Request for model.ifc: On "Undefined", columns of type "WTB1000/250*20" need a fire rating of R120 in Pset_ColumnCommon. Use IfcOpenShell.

First a look at what the model holds.

```python
import ifcopenshell
import ifcopenshell.util.element

model = ifcopenshell.open("model.ifc")
print(model.schema)
storey = next(s for s in model.by_type("IfcBuildingStorey") if s.Name == "Undefined")
columns = [e for e in ifcopenshell.util.element.get_decomposition(storey) if e.is_a("IfcColumn")]
seen = {}
for e in columns:
    element_type = ifcopenshell.util.element.get_type(e)
    key = (element_type.Name if element_type != e and element_type else None, ifcopenshell.util.element.get_pset(e, "Pset_ColumnCommon", "FireRating"))
    seen[key] = seen.get(key, 0) + 1
for (name, value), count in sorted(seen.items(), key=str):
    print(count, "x", name, "|", value)
```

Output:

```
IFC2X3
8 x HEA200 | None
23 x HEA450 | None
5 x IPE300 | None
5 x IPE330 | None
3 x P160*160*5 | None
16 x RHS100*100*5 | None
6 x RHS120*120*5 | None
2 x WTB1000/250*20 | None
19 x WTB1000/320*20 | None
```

```python
import ifcopenshell
import ifcopenshell.api.pset
import ifcopenshell.util.element

model = ifcopenshell.open("model.ifc")

storey = next(s for s in model.by_type("IfcBuildingStorey") if s.Name == "Undefined")
columns = [e for e in ifcopenshell.util.element.get_decomposition(storey) if e.is_a("IfcColumn")]

count = 0
for e in columns:
    element_type = ifcopenshell.util.element.get_type(e)
    if element_type in (None, e) or element_type.Name != "WTB1000/250*20":
        continue
    # add_pset returns the element's existing set when there is one.
    pset = ifcopenshell.api.pset.add_pset(model, product=e, name="Pset_ColumnCommon")
    ifcopenshell.api.pset.edit_pset(model, pset=pset, properties={"FireRating": "R120"})
    count += 1

print(count, "columns updated")

model.write("model_updated.ifc")
```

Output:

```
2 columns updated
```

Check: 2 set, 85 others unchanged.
